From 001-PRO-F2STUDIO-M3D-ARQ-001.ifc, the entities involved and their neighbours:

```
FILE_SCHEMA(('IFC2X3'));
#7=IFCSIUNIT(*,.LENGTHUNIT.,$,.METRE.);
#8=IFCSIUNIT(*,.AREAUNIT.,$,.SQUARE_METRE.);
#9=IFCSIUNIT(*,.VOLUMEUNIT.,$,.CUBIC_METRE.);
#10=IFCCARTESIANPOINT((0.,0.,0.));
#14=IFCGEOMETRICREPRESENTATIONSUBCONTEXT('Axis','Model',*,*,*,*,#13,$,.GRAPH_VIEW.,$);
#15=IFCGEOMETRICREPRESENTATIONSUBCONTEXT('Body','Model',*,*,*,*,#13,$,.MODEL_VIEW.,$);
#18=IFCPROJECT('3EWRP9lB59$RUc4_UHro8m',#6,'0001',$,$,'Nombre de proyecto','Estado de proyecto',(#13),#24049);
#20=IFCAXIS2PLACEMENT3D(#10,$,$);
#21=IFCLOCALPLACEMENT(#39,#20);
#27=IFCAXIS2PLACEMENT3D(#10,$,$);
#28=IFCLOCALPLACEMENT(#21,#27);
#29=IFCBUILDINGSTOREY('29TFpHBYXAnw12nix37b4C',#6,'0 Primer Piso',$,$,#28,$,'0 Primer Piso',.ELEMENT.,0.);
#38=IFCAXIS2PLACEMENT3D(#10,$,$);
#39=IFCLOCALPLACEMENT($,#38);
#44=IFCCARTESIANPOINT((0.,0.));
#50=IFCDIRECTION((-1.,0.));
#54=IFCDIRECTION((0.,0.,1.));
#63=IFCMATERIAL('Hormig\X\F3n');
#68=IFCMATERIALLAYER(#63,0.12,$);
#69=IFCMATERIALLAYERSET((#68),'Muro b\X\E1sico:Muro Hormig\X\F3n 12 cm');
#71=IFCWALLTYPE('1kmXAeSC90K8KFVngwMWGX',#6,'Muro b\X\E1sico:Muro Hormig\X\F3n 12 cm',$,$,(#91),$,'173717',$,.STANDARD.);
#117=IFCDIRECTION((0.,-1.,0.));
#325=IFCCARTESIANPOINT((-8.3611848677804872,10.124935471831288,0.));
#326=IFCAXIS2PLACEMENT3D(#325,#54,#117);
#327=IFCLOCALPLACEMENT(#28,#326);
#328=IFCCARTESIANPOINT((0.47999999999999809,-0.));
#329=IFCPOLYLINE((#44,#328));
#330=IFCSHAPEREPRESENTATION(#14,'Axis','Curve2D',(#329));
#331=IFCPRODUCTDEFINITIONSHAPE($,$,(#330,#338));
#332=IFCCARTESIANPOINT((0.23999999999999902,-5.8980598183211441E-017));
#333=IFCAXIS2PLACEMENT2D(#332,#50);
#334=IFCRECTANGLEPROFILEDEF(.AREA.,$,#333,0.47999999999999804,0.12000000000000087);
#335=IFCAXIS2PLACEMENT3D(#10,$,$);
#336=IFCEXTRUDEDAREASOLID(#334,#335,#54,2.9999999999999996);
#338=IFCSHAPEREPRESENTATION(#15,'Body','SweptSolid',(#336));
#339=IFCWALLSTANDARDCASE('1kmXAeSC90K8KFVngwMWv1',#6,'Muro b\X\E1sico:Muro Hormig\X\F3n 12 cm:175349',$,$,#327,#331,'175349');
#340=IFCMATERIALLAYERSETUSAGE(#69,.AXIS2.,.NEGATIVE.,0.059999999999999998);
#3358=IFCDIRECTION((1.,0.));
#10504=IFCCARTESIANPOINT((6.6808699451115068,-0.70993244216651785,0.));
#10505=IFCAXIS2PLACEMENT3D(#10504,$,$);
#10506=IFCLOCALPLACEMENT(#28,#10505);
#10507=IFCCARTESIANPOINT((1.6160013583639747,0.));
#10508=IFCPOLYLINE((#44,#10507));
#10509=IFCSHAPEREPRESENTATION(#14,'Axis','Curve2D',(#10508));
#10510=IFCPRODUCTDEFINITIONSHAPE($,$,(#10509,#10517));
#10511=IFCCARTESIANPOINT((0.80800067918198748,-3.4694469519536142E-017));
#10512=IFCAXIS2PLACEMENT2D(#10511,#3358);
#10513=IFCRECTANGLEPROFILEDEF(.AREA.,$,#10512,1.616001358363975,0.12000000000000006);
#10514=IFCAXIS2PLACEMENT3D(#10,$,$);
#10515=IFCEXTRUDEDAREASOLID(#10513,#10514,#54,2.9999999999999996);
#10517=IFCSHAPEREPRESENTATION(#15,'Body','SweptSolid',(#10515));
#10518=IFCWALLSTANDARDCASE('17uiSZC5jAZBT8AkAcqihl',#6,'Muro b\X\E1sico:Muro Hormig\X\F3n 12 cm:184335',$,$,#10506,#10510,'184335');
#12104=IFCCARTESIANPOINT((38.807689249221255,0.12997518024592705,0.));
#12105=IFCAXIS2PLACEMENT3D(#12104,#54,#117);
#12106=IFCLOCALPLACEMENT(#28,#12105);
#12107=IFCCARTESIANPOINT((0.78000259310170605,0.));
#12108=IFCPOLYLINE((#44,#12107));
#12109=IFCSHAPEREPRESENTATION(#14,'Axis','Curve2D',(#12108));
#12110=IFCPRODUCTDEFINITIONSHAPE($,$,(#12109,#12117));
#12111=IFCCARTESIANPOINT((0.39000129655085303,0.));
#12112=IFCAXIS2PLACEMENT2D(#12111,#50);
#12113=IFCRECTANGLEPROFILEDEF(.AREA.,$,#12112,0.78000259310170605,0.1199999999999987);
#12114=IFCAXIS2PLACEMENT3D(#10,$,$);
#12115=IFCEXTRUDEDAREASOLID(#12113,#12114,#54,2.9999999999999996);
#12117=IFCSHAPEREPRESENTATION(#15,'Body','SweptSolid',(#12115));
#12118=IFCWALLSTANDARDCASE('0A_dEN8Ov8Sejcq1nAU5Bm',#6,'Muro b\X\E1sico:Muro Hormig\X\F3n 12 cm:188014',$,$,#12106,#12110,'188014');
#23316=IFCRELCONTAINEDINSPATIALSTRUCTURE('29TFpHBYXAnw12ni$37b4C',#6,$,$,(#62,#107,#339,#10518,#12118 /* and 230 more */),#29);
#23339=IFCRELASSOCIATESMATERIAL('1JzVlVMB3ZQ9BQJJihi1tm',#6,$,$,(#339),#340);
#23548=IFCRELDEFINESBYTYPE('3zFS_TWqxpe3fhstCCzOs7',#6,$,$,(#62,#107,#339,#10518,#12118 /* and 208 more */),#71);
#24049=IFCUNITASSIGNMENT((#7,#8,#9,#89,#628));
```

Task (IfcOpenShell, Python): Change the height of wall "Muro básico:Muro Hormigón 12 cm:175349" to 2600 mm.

```python
import ifcopenshell
import ifcopenshell.geom
import ifcopenshell.util.representation
import ifcopenshell.util.shape

model = ifcopenshell.open("001-PRO-F2STUDIO-M3D-ARQ-001.ifc")
settings = ifcopenshell.geom.settings()


def volume(element):
    """Net volume in cubic metres, openings subtracted."""
    shape = ifcopenshell.geom.create_shape(settings, element)
    return ifcopenshell.util.shape.get_volume(shape.geometry)


wall = model.by_guid("1kmXAeSC90K8KFVngwMWv1")
before = volume(wall)

body = ifcopenshell.util.representation.get_representation(wall, "Model", "Body")
solid = body.Items[0]
old_height = solid.Depth
solid.Depth = 2.6
after = volume(wall)

print(f"height {old_height:g} -> {solid.Depth:g}, volume {before:.3f} -> {after:.3f} m3")

model.write("001-PRO-F2STUDIO-M3D-ARQ-001_v2.ifc")
```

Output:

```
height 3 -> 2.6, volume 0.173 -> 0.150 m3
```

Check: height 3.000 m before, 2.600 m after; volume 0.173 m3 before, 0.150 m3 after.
